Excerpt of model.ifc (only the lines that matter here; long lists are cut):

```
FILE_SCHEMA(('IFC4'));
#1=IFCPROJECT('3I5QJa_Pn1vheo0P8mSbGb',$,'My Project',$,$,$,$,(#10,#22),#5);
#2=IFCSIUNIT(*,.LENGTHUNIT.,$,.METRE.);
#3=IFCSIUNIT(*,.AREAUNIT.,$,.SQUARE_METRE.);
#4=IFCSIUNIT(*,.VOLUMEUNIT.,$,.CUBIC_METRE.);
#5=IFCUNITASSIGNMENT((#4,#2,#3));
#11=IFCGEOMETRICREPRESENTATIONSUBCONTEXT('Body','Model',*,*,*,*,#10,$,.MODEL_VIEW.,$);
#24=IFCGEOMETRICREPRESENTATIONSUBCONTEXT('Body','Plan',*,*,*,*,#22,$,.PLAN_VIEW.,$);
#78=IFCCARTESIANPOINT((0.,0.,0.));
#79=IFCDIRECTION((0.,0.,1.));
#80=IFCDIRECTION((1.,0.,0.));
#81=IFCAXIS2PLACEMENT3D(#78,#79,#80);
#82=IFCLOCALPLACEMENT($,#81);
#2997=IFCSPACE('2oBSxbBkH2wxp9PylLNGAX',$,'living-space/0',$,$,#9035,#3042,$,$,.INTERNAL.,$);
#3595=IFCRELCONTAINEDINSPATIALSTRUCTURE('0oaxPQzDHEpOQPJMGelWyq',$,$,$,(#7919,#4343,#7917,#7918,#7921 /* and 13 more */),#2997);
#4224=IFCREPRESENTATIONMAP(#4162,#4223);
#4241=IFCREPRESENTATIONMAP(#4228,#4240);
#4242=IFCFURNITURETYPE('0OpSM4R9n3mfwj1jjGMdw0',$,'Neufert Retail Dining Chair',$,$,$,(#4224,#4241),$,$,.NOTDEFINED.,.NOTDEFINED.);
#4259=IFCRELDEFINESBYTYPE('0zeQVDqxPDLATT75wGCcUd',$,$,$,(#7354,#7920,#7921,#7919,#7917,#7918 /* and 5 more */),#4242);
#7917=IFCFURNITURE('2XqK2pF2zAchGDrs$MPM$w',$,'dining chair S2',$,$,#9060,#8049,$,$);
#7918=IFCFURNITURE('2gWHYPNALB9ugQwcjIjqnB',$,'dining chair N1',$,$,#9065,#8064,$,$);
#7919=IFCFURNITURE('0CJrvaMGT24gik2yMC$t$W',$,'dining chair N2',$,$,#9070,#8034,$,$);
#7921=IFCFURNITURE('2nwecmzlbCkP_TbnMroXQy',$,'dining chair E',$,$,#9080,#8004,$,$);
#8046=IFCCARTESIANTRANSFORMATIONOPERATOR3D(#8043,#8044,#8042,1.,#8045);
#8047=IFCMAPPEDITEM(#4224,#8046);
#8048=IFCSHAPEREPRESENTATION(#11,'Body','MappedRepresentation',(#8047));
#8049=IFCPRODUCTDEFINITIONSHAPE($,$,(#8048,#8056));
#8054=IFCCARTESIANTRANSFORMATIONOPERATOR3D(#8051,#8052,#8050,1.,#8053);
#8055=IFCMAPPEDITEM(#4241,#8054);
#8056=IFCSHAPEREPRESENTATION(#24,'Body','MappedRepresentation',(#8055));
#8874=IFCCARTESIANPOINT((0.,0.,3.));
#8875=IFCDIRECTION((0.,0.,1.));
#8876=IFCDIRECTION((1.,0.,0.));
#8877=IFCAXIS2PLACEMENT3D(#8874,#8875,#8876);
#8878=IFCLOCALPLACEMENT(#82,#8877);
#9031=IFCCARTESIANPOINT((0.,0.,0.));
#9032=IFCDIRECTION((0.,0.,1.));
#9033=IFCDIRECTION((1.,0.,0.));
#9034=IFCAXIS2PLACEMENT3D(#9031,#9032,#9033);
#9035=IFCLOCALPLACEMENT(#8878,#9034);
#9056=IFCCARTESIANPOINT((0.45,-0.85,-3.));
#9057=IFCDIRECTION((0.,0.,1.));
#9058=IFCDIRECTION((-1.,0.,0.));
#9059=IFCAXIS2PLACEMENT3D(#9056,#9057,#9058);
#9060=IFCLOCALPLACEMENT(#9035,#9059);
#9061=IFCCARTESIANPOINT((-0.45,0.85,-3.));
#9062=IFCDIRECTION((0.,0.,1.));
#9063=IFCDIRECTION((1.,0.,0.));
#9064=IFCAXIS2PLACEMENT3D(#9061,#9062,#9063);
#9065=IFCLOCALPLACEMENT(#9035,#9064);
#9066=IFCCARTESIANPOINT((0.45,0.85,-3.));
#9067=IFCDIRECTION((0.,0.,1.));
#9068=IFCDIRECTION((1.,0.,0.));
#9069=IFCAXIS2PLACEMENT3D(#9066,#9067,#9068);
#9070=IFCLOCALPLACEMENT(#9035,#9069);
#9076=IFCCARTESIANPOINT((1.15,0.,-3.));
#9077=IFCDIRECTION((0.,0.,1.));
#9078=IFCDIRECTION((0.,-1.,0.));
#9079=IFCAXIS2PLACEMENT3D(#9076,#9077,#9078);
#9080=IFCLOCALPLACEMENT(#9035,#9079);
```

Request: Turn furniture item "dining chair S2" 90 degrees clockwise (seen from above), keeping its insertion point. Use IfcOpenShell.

```python
import ifcopenshell
import ifcopenshell.api.geometry
import ifcopenshell.util.placement

model = ifcopenshell.open("model.ifc")

item = model.by_guid("2XqK2pF2zAchGDrs$MPM$w")
matrix = ifcopenshell.util.placement.get_local_placement(item.ObjectPlacement)
matrix = matrix @ ifcopenshell.util.placement.rotation(-90, "Z")
ifcopenshell.api.geometry.edit_object_placement(model, product=item, matrix=matrix, is_si=False)

print(ifcopenshell.util.placement.get_local_placement(item.ObjectPlacement).round(3) + 0.0)

model.write("model_edited.ifc")
```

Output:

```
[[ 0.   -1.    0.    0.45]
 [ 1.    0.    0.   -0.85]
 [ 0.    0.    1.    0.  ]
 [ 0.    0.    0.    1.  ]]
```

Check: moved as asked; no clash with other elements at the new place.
